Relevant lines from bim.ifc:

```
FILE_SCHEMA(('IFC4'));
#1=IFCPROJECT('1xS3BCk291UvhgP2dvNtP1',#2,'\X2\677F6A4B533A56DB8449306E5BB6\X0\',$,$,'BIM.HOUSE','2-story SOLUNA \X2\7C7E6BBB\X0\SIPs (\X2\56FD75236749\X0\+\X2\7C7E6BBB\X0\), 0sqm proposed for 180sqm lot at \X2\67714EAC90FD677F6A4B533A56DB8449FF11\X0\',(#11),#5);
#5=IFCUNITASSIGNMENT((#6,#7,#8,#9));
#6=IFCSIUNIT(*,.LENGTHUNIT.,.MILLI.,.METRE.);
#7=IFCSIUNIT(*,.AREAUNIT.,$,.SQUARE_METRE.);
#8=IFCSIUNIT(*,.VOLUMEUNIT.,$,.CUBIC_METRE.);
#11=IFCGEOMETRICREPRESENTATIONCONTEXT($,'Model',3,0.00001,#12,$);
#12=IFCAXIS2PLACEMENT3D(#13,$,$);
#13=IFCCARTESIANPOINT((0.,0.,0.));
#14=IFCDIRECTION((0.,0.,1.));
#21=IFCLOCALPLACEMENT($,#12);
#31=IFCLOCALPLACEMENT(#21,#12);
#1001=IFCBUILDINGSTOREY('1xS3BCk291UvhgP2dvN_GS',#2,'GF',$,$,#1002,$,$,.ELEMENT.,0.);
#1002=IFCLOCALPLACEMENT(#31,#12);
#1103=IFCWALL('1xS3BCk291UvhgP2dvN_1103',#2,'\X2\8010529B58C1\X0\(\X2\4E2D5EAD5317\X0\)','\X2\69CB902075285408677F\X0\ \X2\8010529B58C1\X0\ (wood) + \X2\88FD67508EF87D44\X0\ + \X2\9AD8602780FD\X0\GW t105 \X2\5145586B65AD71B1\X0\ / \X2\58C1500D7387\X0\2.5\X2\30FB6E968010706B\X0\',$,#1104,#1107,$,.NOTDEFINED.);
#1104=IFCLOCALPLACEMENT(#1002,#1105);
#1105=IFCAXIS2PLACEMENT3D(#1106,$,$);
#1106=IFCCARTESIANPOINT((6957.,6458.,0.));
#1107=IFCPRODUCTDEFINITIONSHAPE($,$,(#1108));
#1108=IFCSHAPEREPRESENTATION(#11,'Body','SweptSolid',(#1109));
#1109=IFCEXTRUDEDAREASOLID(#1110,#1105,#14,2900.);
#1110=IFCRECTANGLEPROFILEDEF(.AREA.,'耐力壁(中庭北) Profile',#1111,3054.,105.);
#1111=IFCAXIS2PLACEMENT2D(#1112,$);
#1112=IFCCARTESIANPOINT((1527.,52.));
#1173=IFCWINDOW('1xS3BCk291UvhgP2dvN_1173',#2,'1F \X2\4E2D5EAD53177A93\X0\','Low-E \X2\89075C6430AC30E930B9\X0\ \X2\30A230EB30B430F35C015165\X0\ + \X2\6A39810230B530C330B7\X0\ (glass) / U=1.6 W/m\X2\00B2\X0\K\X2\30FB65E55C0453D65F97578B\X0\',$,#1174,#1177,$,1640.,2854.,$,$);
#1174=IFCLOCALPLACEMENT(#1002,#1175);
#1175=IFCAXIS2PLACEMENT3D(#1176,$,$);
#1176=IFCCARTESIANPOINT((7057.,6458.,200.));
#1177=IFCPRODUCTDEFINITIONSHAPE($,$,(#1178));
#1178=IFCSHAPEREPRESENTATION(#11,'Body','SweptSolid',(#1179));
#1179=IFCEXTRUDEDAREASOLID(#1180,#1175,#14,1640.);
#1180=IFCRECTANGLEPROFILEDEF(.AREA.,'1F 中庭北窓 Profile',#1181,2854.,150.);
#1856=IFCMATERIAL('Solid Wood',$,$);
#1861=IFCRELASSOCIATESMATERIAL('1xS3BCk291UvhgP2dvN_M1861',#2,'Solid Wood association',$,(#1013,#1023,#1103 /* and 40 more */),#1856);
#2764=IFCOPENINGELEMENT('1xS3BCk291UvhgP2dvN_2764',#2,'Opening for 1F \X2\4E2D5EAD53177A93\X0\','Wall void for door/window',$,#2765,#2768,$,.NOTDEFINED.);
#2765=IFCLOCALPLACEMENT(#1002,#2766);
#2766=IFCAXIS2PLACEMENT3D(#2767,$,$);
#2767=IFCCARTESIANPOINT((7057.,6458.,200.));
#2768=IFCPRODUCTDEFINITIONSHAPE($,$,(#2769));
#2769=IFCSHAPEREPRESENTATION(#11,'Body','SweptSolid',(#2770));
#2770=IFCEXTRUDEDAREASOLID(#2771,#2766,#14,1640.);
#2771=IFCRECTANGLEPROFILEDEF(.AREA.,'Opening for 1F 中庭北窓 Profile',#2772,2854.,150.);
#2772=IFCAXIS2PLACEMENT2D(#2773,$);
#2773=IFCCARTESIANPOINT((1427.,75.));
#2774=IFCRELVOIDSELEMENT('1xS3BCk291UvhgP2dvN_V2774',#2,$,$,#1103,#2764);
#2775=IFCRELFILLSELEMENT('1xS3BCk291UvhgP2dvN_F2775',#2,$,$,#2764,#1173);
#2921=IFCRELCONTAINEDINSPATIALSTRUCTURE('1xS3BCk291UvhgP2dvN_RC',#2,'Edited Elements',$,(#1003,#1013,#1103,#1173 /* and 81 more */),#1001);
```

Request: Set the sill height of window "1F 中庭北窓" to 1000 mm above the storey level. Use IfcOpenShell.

```python
import numpy as np
import ifcopenshell
import ifcopenshell.api.geometry
import ifcopenshell.geom
import ifcopenshell.util.element
import ifcopenshell.util.placement
import ifcopenshell.util.shape
import ifcopenshell.util.unit

model = ifcopenshell.open("bim.ifc")
unit_scale = ifcopenshell.util.unit.calculate_unit_scale(model)

window = model.by_guid("1xS3BCk291UvhgP2dvN_1173")
opening = window.FillsVoids[0].RelatingOpeningElement
storey = ifcopenshell.util.element.get_container(window, ifc_class="IfcBuildingStorey")
level = ifcopenshell.util.placement.get_local_placement(storey.ObjectPlacement)[2, 3]

# The opening's origin need not be at the sill, so measure its lowest point.
shape = ifcopenshell.geom.create_shape(ifcopenshell.geom.settings(), opening)
bottom = ifcopenshell.util.shape.get_shape_bottom_elevation(shape, shape.geometry) / unit_scale
dz = level + 1 / unit_scale - bottom

shift = np.array([0.0, 0.0, dz])
# The window is not placed relative to its opening, so move both.
for product in (opening, window):
    matrix = ifcopenshell.util.placement.get_local_placement(product.ObjectPlacement)
    matrix[:3, 3] += shift
    ifcopenshell.api.geometry.edit_object_placement(model, product=product, matrix=matrix, is_si=False)

print(f"moved by {dz * unit_scale:+.3f} m")

model.write("bim-out.ifc")
```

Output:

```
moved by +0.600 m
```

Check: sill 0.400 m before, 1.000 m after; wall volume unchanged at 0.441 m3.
